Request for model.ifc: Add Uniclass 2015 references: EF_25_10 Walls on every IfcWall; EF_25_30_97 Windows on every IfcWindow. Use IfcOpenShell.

First a look at what the model holds.

```python
import ifcopenshell

model = ifcopenshell.open("model.ifc")
print(model.schema)
print("classifications:", [c.Name for c in model.by_type("IfcClassification")])
for ifc_class in ("IfcDoor", "IfcRoof", "IfcStair", "IfcWall", "IfcWindow"):
    print(ifc_class, len(model.by_type(ifc_class)))
```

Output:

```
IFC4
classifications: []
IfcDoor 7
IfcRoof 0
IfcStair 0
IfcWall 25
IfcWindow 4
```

```python
import ifcopenshell
import ifcopenshell.api.classification

model = ifcopenshell.open("model.ifc")

system = ifcopenshell.api.classification.add_classification(model, classification="Uniclass 2015")

codes = {
    "IfcWall": ("EF_25_10", "Walls"),
    "IfcWindow": ("EF_25_30_97", "Windows"),
}
for ifc_class, (code, name) in codes.items():
    products = model.by_type(ifc_class)
    ifcopenshell.api.classification.add_reference(
        model, products=products, classification=system, identification=code, name=name
    )
    print(code, len(products))

model.write("model_updated.ifc")
```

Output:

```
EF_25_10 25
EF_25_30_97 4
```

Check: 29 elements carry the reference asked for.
